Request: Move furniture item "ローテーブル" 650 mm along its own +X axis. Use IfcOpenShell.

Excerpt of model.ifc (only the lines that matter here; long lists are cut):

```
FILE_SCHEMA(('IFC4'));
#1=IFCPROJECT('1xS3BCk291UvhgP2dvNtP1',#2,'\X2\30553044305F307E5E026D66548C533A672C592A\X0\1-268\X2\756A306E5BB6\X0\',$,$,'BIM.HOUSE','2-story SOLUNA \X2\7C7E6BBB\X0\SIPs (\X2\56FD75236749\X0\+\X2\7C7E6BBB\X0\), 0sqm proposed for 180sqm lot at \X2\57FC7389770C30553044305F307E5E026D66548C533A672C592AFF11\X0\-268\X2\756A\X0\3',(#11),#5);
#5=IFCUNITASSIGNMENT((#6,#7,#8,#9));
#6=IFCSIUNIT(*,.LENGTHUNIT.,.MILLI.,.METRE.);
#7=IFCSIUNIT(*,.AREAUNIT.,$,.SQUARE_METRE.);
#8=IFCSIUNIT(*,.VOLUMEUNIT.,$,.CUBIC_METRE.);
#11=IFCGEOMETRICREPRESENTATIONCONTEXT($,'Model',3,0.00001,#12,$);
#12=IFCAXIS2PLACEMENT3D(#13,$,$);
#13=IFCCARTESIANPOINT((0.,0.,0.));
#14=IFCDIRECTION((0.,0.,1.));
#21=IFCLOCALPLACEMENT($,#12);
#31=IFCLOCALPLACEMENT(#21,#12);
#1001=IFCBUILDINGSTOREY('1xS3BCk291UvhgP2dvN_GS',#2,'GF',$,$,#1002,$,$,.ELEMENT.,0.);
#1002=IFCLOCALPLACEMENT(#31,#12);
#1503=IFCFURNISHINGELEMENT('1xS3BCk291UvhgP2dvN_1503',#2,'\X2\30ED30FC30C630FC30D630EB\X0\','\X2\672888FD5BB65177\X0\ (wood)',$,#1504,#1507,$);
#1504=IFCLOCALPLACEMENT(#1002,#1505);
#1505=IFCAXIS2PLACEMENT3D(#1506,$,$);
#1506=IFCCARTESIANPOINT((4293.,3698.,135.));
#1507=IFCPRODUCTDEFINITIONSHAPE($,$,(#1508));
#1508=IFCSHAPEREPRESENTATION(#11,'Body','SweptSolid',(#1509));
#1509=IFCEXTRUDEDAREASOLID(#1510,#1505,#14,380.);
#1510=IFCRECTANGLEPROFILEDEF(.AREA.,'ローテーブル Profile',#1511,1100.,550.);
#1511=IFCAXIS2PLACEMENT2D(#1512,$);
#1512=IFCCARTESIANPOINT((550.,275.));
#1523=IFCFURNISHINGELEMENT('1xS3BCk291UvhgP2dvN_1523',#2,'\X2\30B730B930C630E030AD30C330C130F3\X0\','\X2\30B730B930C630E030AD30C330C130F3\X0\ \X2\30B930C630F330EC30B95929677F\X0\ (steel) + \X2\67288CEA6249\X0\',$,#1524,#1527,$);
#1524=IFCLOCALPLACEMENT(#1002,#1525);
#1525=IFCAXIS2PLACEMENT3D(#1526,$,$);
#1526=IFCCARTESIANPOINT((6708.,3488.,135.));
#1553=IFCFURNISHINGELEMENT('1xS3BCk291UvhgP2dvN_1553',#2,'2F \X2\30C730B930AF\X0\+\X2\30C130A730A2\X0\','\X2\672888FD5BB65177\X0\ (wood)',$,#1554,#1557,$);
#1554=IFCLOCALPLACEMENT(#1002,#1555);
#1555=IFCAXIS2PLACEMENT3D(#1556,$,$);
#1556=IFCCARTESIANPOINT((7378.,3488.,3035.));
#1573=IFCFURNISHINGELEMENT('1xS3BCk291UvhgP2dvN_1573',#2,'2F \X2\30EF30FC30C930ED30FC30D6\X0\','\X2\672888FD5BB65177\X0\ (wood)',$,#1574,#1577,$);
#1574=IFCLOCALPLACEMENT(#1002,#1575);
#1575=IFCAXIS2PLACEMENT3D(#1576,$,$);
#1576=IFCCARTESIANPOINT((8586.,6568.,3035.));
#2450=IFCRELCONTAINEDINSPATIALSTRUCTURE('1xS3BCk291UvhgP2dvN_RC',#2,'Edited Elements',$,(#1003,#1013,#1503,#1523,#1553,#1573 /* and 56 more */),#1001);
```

```python
import ifcopenshell
import ifcopenshell.api.geometry
import ifcopenshell.util.placement

model = ifcopenshell.open("model.ifc")

item = model.by_guid("1xS3BCk291UvhgP2dvN_1503")
matrix = ifcopenshell.util.placement.get_local_placement(item.ObjectPlacement)
matrix[:3, 3] += matrix[:3, 0] * 650.0
ifcopenshell.api.geometry.edit_object_placement(model, product=item, matrix=matrix, is_si=False)

print(ifcopenshell.util.placement.get_local_placement(item.ObjectPlacement).round(3) + 0.0)

model.write("model_v2.ifc")
```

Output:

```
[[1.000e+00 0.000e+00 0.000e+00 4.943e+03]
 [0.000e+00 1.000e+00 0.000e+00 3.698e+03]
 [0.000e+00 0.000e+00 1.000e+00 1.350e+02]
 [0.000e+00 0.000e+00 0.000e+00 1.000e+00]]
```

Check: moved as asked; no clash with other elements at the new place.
